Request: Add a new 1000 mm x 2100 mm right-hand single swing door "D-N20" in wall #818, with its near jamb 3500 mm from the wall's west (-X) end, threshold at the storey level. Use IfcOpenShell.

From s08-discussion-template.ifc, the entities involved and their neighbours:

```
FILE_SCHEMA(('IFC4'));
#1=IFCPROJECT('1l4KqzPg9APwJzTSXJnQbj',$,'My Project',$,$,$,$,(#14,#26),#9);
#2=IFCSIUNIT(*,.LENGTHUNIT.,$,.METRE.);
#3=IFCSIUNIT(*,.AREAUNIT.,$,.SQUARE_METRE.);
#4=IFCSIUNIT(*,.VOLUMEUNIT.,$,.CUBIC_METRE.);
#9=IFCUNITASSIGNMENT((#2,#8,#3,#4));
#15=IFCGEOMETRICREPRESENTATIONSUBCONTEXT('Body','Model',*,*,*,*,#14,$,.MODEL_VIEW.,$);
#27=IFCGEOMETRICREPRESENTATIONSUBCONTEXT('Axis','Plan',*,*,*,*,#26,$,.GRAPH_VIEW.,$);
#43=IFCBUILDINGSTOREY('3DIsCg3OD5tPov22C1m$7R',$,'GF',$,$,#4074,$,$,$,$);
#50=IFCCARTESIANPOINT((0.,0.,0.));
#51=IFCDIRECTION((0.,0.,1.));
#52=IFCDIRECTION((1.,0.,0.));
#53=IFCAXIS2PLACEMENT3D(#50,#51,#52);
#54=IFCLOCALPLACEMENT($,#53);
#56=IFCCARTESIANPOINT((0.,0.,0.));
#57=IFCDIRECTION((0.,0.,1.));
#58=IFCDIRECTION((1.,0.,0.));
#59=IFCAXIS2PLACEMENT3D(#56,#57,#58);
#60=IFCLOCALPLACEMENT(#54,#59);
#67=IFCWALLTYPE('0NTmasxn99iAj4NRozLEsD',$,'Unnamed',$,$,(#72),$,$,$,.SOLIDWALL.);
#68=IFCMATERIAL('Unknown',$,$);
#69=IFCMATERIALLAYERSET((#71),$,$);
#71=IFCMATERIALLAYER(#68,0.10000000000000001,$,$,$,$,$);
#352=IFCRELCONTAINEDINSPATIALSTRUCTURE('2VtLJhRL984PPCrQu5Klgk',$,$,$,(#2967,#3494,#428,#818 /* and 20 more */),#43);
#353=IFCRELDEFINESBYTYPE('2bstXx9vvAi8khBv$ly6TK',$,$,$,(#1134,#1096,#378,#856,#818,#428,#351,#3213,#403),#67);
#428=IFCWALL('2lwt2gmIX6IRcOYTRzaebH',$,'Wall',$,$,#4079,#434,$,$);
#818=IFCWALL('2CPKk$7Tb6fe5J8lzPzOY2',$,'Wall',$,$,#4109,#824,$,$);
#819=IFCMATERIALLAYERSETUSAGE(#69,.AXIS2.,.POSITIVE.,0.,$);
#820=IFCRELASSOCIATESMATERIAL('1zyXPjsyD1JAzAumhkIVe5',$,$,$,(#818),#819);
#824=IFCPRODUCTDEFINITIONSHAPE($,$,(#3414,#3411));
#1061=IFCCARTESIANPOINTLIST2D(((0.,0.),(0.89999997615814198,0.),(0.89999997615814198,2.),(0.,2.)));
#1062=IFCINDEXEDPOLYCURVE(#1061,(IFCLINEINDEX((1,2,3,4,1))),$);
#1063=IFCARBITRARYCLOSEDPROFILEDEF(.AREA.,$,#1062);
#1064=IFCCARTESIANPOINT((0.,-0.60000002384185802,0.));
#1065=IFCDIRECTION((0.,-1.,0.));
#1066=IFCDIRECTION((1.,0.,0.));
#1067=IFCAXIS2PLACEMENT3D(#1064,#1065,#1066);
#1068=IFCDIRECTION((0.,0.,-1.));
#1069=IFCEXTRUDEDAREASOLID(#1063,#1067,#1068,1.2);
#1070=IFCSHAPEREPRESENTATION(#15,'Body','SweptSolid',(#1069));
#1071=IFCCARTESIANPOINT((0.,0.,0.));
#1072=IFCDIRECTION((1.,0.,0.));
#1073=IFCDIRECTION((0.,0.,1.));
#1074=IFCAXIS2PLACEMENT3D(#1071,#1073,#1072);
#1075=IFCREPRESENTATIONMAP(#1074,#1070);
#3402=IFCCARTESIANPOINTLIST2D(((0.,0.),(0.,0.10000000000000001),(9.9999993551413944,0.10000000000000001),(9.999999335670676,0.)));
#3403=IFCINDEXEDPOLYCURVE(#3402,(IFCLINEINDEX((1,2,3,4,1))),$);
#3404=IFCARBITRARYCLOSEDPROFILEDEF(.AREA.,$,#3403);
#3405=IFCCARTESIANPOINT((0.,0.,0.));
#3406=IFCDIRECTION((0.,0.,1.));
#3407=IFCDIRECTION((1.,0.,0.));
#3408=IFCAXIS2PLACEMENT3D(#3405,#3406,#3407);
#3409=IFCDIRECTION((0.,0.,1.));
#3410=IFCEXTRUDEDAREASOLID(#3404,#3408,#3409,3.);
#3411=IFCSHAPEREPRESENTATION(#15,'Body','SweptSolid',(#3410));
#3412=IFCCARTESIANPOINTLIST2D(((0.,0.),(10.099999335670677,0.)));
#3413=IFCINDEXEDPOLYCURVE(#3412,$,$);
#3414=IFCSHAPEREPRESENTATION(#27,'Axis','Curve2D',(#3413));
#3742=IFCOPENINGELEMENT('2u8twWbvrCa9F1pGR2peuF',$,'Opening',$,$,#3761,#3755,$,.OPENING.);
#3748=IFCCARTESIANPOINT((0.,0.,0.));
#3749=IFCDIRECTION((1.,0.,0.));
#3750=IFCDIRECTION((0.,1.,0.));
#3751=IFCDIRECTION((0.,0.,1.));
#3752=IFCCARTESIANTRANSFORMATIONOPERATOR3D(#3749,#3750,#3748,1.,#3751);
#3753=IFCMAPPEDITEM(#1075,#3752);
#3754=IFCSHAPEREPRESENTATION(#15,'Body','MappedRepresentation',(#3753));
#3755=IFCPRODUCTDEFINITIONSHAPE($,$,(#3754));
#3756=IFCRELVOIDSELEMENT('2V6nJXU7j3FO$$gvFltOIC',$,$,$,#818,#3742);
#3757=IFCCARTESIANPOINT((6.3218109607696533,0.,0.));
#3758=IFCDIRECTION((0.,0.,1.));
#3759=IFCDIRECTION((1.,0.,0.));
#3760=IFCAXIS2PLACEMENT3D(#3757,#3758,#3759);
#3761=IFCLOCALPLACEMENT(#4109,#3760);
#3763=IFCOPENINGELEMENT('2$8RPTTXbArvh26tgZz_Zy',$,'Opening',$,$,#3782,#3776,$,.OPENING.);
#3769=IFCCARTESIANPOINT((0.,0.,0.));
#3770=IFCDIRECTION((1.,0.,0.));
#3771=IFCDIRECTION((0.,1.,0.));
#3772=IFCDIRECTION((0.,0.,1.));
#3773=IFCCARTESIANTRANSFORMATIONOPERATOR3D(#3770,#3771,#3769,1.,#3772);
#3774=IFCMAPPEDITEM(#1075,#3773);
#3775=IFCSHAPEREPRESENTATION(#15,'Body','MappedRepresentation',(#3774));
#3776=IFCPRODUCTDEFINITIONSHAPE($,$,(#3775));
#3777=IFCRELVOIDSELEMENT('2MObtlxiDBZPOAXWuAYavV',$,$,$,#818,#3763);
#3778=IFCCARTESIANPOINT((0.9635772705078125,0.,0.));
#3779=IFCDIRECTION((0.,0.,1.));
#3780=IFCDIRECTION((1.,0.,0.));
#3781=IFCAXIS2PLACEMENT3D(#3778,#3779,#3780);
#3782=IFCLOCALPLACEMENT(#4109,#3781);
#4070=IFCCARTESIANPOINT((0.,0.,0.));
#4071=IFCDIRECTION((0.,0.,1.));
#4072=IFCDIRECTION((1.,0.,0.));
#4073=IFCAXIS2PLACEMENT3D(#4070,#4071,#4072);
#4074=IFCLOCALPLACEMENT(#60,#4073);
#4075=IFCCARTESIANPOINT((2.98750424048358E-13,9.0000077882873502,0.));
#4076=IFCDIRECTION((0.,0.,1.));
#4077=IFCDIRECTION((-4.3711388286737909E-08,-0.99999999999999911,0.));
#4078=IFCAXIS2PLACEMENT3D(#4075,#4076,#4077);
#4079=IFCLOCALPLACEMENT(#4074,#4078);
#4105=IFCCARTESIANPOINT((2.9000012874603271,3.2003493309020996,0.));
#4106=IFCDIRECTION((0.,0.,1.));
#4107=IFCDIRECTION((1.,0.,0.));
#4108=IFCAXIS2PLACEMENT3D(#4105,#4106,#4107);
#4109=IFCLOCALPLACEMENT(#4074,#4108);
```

```python
import numpy as np
import ifcopenshell
import ifcopenshell.api.feature
import ifcopenshell.api.geometry
import ifcopenshell.api.root
import ifcopenshell.api.spatial
import ifcopenshell.geom
import ifcopenshell.util.element
import ifcopenshell.util.placement
import ifcopenshell.util.representation
import ifcopenshell.util.shape
import ifcopenshell.util.unit

model = ifcopenshell.open("s08-discussion-template.ifc")
unit_scale = ifcopenshell.util.unit.calculate_unit_scale(model)
settings = ifcopenshell.geom.settings()


def volume(element):
    """Net volume in cubic metres, openings subtracted."""
    shape = ifcopenshell.geom.create_shape(settings, element)
    return ifcopenshell.util.shape.get_volume(shape.geometry)


wall = model.by_guid("2CPKk$7Tb6fe5J8lzPzOY2")
storey = ifcopenshell.util.element.get_container(wall, ifc_class="IfcBuildingStorey")
context = ifcopenshell.util.representation.get_context(model, "Model", "Body", "MODEL_VIEW")
before = volume(wall)

width, height, from_end, sill = 1, 2.1, 3.5, 0.0  # metres

# The wall runs along its own X axis, and the end named is its -X end.
wall_shape = ifcopenshell.geom.create_shape(settings, wall)
x, y, z = ifcopenshell.util.shape.get_vertices(wall_shape.geometry).T
start = x.min() + from_end
face, thickness = float(y.min()), float(y.max() - y.min())
wall_matrix = ifcopenshell.util.placement.get_local_placement(wall.ObjectPlacement)
level = ifcopenshell.util.placement.get_local_placement(storey.ObjectPlacement)[2, 3]


def in_wall(x, y):
    """Placement at x, y metres in the wall's axes, at sill height."""
    matrix = wall_matrix.copy()
    matrix[:, 3] = wall_matrix @ np.array([x / unit_scale, y / unit_scale, 0.0, 1.0])
    matrix[2, 3] = level + sill / unit_scale
    return matrix


# Opening: a box that overshoots both wall faces by 50 mm.
opening = ifcopenshell.api.root.create_entity(model, ifc_class="IfcOpeningElement", predefined_type="OPENING")
box = ifcopenshell.api.geometry.add_wall_representation(
    model, context=context, length=width, height=height, thickness=thickness + 0.1
)
ifcopenshell.api.geometry.assign_representation(model, product=opening, representation=box)
ifcopenshell.api.geometry.edit_object_placement(model, product=opening, matrix=in_wall(start, face - 0.05), is_si=False)
ifcopenshell.api.feature.add_feature(model, feature=opening, element=wall)

door = ifcopenshell.api.root.create_entity(model, ifc_class="IfcDoor", name="D-N20", predefined_type="DOOR")
door.OverallWidth, door.OverallHeight = width / unit_scale, height / unit_scale
door.OperationType = "SINGLE_SWING_RIGHT"
body = ifcopenshell.api.geometry.add_door_representation(
    model,
    context=context,
    overall_width=door.OverallWidth,
    overall_height=door.OverallHeight,
    operation_type="SINGLE_SWING_RIGHT",
    lining_properties={"LiningDepth": thickness / unit_scale, "ThresholdDepth": thickness / unit_scale},
)
ifcopenshell.api.geometry.assign_representation(model, product=door, representation=body)
ifcopenshell.api.spatial.assign_container(model, products=[door], relating_structure=storey)
ifcopenshell.api.feature.add_filling(model, opening=opening, element=door)

# The lining spans the wall, so the door starts at the wall face.
ifcopenshell.api.geometry.edit_object_placement(model, product=door, matrix=in_wall(start, face), is_si=False)

after = volume(wall)

print(f"wall volume {before:.3f} -> {after:.3f} m3")

model.write("s08-discussion-template_edited.ifc")
```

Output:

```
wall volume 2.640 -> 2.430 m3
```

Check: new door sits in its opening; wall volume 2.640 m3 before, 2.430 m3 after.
